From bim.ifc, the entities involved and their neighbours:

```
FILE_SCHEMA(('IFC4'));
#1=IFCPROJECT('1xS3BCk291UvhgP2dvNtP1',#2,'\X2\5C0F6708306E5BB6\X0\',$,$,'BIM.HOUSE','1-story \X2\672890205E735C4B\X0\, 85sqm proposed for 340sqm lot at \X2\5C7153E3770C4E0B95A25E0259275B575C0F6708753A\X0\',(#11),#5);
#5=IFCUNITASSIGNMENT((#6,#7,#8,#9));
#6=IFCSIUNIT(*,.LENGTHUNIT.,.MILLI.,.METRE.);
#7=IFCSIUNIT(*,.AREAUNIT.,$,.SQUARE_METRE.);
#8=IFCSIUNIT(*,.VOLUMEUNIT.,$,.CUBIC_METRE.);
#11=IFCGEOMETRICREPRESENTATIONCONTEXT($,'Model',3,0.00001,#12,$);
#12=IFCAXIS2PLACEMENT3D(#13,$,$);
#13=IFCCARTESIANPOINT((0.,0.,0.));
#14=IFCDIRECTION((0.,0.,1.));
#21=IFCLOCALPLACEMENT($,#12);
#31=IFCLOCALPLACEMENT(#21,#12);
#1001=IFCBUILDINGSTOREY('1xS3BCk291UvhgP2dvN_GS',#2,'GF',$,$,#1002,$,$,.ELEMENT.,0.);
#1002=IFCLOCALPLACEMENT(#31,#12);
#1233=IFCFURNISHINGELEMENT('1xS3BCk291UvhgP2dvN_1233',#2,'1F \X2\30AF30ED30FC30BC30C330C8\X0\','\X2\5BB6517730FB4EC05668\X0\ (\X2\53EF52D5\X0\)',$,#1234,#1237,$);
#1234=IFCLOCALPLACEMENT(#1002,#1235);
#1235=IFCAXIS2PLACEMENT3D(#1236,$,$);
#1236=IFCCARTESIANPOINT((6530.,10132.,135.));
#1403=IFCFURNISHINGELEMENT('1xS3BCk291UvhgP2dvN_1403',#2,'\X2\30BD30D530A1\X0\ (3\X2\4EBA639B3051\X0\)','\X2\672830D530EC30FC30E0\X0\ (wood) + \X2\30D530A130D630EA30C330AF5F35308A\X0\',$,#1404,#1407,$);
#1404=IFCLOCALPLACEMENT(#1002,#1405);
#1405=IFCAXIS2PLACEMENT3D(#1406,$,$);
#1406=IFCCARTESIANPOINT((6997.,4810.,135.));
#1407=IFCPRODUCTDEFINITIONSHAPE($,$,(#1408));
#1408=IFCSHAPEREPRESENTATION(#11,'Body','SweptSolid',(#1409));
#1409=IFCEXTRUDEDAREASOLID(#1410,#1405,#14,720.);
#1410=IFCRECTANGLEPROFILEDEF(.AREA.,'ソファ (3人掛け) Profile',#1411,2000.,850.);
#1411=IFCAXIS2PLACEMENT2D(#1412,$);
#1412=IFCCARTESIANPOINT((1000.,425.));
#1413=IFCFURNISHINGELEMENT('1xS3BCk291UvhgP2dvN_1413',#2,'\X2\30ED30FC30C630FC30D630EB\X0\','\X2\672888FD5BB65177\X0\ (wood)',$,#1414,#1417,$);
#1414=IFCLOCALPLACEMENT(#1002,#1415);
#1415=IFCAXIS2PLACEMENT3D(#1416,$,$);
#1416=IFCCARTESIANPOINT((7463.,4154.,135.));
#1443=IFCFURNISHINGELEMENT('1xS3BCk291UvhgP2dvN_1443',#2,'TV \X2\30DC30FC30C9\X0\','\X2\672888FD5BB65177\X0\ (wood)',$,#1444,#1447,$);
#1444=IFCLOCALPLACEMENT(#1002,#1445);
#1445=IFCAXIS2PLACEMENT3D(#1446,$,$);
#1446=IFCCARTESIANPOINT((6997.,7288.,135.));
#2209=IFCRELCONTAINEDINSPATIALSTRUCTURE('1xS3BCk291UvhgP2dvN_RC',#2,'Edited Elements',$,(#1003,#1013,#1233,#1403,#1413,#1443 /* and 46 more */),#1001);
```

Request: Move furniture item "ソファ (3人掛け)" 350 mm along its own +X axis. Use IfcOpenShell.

```python
import ifcopenshell
import ifcopenshell.api.geometry
import ifcopenshell.util.placement
import ifcopenshell.util.unit

model = ifcopenshell.open("bim.ifc")
unit_scale = ifcopenshell.util.unit.calculate_unit_scale(model)

item = model.by_id(1403)
matrix = ifcopenshell.util.placement.get_local_placement(item.ObjectPlacement)
matrix[:3, 3] += matrix[:3, 0] * 0.35 / unit_scale
ifcopenshell.api.geometry.edit_object_placement(model, product=item, matrix=matrix, is_si=False)

print(ifcopenshell.util.placement.get_local_placement(item.ObjectPlacement).round(3) + 0.0)

model.write("bim_rev.ifc")
```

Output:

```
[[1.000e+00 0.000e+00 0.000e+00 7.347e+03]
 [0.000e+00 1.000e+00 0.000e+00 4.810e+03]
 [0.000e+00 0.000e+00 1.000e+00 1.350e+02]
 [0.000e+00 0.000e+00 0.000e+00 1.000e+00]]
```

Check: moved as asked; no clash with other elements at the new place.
